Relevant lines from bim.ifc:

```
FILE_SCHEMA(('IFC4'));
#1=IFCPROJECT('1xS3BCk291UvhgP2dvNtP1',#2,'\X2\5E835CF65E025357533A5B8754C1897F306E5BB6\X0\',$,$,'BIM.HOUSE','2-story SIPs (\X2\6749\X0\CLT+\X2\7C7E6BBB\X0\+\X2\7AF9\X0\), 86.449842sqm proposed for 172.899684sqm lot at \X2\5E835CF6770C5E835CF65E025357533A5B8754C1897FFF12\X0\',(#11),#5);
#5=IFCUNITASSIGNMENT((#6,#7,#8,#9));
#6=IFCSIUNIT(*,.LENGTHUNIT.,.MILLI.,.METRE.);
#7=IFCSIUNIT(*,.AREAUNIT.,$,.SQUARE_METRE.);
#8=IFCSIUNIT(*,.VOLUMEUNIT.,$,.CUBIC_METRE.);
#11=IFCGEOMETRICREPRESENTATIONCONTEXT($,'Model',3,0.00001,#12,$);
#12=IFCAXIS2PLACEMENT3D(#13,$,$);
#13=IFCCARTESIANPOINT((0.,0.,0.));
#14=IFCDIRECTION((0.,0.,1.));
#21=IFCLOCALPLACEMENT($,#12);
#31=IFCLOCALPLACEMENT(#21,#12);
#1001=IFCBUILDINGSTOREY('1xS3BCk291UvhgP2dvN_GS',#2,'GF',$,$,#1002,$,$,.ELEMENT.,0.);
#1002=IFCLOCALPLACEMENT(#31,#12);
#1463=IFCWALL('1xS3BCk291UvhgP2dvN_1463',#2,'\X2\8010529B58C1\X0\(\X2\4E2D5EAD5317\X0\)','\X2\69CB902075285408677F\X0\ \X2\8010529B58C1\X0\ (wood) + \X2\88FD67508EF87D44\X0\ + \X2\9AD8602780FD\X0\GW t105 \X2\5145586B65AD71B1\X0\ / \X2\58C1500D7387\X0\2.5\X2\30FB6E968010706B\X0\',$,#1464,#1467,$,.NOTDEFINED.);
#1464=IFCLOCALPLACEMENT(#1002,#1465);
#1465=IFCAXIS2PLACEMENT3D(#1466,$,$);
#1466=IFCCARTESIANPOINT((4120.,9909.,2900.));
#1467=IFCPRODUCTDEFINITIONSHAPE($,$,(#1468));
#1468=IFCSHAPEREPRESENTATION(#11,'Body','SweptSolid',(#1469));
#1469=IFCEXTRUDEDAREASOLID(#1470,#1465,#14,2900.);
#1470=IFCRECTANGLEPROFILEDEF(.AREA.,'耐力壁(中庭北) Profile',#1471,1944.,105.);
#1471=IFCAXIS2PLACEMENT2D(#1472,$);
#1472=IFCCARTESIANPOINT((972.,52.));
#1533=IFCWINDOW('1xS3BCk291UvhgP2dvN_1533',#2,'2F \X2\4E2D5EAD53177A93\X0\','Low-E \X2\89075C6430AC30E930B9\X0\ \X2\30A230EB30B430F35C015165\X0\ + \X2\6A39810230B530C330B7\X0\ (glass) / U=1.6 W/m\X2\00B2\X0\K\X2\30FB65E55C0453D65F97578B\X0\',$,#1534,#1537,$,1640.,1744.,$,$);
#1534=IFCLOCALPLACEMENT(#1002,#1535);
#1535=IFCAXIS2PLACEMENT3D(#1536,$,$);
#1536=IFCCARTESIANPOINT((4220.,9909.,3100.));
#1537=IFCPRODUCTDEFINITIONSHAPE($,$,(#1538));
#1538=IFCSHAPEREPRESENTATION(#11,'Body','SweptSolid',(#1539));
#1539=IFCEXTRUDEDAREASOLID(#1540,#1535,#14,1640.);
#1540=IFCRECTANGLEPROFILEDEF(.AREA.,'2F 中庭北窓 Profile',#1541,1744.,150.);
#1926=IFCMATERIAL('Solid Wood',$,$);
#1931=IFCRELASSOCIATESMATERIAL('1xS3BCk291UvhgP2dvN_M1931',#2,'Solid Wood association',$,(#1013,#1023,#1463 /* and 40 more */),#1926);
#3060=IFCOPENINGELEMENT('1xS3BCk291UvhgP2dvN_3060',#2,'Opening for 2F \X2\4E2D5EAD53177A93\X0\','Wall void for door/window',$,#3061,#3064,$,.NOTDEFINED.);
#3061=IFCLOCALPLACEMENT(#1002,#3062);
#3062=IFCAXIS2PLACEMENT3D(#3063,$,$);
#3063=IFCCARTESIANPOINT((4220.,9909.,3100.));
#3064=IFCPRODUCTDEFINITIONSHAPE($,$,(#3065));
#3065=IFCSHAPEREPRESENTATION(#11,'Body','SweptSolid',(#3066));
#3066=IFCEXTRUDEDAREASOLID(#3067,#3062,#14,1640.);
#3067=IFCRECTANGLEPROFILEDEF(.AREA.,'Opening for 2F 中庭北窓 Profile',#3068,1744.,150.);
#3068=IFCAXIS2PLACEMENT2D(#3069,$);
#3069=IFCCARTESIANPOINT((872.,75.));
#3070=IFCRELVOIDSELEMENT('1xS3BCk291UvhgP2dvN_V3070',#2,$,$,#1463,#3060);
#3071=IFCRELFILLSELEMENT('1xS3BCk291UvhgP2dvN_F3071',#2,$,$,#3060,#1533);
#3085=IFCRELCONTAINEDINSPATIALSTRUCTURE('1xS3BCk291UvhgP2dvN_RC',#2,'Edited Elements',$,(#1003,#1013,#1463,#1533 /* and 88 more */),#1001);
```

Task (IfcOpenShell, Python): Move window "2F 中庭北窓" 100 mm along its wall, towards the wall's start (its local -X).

```python
import ifcopenshell
import ifcopenshell.api.geometry
import ifcopenshell.util.placement
import ifcopenshell.util.unit

model = ifcopenshell.open("bim.ifc")
unit_scale = ifcopenshell.util.unit.calculate_unit_scale(model)

window = model.by_id(1533)
opening = window.FillsVoids[0].RelatingOpeningElement
wall = opening.VoidsElements[0].RelatingBuildingElement

wall_matrix = ifcopenshell.util.placement.get_local_placement(wall.ObjectPlacement)
shift = wall_matrix[:3, 0] * -0.1 / unit_scale
before = ifcopenshell.util.placement.get_local_placement(window.ObjectPlacement)[:3, 3].copy()

# The window is not placed relative to its opening, so move both.
for product in (opening, window):
    matrix = ifcopenshell.util.placement.get_local_placement(product.ObjectPlacement)
    matrix[:3, 3] += shift
    ifcopenshell.api.geometry.edit_object_placement(model, product=product, matrix=matrix, is_si=False)

after = ifcopenshell.util.placement.get_local_placement(window.ObjectPlacement)[:3, 3]
print("window moved by", (after - before).round(3) + 0.0)

model.write("bim_rev.ifc")
```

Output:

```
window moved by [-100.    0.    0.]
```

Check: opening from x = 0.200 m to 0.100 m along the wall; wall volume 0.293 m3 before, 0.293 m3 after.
